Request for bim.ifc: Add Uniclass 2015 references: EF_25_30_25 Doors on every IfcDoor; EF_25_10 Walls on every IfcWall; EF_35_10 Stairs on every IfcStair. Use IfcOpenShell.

First a look at what the model holds.

```python
import ifcopenshell

model = ifcopenshell.open("bim.ifc")
print(model.schema)
print("classifications:", [c.Name for c in model.by_type("IfcClassification")])
for ifc_class in ("IfcDoor", "IfcRoof", "IfcStair", "IfcWall", "IfcWindow"):
    print(ifc_class, len(model.by_type(ifc_class)))
```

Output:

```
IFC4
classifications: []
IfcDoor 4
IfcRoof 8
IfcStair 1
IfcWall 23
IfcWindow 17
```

```python
import ifcopenshell
import ifcopenshell.api.classification

model = ifcopenshell.open("bim.ifc")

system = ifcopenshell.api.classification.add_classification(model, classification="Uniclass 2015")

codes = {
    "IfcDoor": ("EF_25_30_25", "Doors"),
    "IfcWall": ("EF_25_10", "Walls"),
    "IfcStair": ("EF_35_10", "Stairs"),
}
for ifc_class, (code, name) in codes.items():
    products = model.by_type(ifc_class)
    ifcopenshell.api.classification.add_reference(
        model, products=products, classification=system, identification=code, name=name
    )
    print(code, len(products))

model.write("bim_rev.ifc")
```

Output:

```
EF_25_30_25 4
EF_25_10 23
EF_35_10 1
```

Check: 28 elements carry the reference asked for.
